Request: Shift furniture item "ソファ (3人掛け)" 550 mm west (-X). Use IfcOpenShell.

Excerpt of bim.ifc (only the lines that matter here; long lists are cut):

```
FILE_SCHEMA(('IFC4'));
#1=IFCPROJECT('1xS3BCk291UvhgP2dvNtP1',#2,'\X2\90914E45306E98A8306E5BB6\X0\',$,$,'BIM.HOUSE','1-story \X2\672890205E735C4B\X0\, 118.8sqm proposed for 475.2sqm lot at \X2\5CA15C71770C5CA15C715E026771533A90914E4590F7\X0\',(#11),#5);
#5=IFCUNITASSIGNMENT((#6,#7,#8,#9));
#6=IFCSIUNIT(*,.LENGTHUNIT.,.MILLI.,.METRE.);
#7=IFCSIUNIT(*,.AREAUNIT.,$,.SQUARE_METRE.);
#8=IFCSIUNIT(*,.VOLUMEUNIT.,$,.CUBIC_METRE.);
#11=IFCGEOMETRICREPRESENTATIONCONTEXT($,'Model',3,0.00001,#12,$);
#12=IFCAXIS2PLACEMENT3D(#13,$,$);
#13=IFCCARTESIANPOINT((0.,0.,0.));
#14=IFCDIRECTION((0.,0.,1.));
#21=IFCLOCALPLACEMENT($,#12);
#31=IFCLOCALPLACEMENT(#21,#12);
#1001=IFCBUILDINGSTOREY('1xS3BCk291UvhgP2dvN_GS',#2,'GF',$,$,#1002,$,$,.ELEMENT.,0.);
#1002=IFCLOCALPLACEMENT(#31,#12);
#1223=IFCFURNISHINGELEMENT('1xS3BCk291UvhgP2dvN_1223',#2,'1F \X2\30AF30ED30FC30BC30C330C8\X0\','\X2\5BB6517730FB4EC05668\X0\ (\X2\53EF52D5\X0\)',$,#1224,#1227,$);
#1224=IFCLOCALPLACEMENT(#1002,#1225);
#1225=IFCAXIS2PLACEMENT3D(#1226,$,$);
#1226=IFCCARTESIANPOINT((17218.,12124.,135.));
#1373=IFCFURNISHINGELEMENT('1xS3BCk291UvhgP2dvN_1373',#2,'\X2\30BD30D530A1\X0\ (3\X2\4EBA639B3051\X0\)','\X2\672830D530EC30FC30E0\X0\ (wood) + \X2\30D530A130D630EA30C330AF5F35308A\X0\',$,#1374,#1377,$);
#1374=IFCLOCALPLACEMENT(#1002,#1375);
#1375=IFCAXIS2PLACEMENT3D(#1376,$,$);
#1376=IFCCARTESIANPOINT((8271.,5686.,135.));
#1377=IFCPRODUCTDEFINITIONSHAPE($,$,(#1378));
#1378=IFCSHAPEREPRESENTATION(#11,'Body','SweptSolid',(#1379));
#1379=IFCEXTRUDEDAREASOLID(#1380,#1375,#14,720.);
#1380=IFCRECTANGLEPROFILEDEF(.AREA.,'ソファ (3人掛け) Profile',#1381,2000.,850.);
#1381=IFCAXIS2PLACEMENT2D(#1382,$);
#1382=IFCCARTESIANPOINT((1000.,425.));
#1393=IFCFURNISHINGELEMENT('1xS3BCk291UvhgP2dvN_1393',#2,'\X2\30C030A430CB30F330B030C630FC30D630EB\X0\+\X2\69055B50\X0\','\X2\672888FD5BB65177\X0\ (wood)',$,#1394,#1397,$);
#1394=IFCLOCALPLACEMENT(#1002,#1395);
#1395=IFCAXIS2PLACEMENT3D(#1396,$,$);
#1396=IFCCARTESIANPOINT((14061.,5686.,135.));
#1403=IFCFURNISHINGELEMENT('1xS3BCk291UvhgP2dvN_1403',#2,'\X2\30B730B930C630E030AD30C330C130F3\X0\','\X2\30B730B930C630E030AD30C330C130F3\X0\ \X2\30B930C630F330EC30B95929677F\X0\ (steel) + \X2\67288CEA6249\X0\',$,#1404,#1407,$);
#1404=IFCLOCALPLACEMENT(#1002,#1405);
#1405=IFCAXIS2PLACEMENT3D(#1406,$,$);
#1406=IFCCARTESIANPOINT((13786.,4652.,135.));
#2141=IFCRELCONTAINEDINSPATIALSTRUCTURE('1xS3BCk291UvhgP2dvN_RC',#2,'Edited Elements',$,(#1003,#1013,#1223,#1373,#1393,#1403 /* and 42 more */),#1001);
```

```python
import ifcopenshell
import ifcopenshell.api.geometry
import ifcopenshell.util.placement
import ifcopenshell.util.unit

model = ifcopenshell.open("bim.ifc")
unit_scale = ifcopenshell.util.unit.calculate_unit_scale(model)

item = model.by_guid("1xS3BCk291UvhgP2dvN_1373")
matrix = ifcopenshell.util.placement.get_local_placement(item.ObjectPlacement)
matrix[0, 3] -= 0.55 / unit_scale
ifcopenshell.api.geometry.edit_object_placement(model, product=item, matrix=matrix, is_si=False)

print(ifcopenshell.util.placement.get_local_placement(item.ObjectPlacement).round(3) + 0.0)

model.write("bim_edited.ifc")
```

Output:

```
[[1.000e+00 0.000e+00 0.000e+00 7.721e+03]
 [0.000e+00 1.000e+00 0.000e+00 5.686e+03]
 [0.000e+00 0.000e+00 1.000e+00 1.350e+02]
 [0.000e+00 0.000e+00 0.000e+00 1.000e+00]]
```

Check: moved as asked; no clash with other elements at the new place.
